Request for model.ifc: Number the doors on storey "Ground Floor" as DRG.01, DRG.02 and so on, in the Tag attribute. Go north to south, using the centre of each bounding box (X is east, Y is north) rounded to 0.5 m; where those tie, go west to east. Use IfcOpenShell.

First a look at what the model holds.

```python
import ifcopenshell
import ifcopenshell.util.element
import ifcopenshell.util.placement

model = ifcopenshell.open("model.ifc")
print(model.schema)
storey = next(s for s in model.by_type("IfcBuildingStorey") if s.Name == "Ground Floor")
doors = [e for e in ifcopenshell.util.element.get_decomposition(storey) if e.is_a("IfcDoor")]
for e in sorted(doors, key=lambda e: e.id()):
    origin = ifcopenshell.util.placement.get_local_placement(e.ObjectPlacement)[:3, 3]
    print(e.id(), e.Tag, e.Name, origin.round(2) + 0.0, sep=" | ")
```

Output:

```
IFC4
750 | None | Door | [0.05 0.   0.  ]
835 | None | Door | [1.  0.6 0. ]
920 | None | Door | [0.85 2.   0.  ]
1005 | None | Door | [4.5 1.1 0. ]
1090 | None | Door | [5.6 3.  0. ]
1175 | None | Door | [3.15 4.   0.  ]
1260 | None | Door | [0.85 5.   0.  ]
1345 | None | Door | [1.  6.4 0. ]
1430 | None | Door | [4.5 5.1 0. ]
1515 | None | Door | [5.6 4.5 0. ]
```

```python
import ifcopenshell
import ifcopenshell.geom
import ifcopenshell.util.element
import ifcopenshell.util.shape

model = ifcopenshell.open("model.ifc")
settings = ifcopenshell.geom.settings()
settings.set("use-world-coords", True)


def centre(element):
    shape = ifcopenshell.geom.create_shape(settings, element)
    return ifcopenshell.util.shape.get_bbox_centroid(shape.geometry)


storey = next(s for s in model.by_type("IfcBuildingStorey") if s.Name == "Ground Floor")
doors = [e for e in ifcopenshell.util.element.get_decomposition(storey) if e.is_a("IfcDoor")]

# Insertion points can sit at a corner or the storey origin, so sort by the geometry (in metres).
centres = {e: centre(e) for e in doors}
doors.sort(key=lambda e: (-round(centres[e][1] / 0.5), centres[e][0]))

for i, e in enumerate(doors, start=1):
    number = f"DRG.{i:02d}"
    e.Tag = number
    print(e.id(), number)

model.write("model_v2.ifc")
```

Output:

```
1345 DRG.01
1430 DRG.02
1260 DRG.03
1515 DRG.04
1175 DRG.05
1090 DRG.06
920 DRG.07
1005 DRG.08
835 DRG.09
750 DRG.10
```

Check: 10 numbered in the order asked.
